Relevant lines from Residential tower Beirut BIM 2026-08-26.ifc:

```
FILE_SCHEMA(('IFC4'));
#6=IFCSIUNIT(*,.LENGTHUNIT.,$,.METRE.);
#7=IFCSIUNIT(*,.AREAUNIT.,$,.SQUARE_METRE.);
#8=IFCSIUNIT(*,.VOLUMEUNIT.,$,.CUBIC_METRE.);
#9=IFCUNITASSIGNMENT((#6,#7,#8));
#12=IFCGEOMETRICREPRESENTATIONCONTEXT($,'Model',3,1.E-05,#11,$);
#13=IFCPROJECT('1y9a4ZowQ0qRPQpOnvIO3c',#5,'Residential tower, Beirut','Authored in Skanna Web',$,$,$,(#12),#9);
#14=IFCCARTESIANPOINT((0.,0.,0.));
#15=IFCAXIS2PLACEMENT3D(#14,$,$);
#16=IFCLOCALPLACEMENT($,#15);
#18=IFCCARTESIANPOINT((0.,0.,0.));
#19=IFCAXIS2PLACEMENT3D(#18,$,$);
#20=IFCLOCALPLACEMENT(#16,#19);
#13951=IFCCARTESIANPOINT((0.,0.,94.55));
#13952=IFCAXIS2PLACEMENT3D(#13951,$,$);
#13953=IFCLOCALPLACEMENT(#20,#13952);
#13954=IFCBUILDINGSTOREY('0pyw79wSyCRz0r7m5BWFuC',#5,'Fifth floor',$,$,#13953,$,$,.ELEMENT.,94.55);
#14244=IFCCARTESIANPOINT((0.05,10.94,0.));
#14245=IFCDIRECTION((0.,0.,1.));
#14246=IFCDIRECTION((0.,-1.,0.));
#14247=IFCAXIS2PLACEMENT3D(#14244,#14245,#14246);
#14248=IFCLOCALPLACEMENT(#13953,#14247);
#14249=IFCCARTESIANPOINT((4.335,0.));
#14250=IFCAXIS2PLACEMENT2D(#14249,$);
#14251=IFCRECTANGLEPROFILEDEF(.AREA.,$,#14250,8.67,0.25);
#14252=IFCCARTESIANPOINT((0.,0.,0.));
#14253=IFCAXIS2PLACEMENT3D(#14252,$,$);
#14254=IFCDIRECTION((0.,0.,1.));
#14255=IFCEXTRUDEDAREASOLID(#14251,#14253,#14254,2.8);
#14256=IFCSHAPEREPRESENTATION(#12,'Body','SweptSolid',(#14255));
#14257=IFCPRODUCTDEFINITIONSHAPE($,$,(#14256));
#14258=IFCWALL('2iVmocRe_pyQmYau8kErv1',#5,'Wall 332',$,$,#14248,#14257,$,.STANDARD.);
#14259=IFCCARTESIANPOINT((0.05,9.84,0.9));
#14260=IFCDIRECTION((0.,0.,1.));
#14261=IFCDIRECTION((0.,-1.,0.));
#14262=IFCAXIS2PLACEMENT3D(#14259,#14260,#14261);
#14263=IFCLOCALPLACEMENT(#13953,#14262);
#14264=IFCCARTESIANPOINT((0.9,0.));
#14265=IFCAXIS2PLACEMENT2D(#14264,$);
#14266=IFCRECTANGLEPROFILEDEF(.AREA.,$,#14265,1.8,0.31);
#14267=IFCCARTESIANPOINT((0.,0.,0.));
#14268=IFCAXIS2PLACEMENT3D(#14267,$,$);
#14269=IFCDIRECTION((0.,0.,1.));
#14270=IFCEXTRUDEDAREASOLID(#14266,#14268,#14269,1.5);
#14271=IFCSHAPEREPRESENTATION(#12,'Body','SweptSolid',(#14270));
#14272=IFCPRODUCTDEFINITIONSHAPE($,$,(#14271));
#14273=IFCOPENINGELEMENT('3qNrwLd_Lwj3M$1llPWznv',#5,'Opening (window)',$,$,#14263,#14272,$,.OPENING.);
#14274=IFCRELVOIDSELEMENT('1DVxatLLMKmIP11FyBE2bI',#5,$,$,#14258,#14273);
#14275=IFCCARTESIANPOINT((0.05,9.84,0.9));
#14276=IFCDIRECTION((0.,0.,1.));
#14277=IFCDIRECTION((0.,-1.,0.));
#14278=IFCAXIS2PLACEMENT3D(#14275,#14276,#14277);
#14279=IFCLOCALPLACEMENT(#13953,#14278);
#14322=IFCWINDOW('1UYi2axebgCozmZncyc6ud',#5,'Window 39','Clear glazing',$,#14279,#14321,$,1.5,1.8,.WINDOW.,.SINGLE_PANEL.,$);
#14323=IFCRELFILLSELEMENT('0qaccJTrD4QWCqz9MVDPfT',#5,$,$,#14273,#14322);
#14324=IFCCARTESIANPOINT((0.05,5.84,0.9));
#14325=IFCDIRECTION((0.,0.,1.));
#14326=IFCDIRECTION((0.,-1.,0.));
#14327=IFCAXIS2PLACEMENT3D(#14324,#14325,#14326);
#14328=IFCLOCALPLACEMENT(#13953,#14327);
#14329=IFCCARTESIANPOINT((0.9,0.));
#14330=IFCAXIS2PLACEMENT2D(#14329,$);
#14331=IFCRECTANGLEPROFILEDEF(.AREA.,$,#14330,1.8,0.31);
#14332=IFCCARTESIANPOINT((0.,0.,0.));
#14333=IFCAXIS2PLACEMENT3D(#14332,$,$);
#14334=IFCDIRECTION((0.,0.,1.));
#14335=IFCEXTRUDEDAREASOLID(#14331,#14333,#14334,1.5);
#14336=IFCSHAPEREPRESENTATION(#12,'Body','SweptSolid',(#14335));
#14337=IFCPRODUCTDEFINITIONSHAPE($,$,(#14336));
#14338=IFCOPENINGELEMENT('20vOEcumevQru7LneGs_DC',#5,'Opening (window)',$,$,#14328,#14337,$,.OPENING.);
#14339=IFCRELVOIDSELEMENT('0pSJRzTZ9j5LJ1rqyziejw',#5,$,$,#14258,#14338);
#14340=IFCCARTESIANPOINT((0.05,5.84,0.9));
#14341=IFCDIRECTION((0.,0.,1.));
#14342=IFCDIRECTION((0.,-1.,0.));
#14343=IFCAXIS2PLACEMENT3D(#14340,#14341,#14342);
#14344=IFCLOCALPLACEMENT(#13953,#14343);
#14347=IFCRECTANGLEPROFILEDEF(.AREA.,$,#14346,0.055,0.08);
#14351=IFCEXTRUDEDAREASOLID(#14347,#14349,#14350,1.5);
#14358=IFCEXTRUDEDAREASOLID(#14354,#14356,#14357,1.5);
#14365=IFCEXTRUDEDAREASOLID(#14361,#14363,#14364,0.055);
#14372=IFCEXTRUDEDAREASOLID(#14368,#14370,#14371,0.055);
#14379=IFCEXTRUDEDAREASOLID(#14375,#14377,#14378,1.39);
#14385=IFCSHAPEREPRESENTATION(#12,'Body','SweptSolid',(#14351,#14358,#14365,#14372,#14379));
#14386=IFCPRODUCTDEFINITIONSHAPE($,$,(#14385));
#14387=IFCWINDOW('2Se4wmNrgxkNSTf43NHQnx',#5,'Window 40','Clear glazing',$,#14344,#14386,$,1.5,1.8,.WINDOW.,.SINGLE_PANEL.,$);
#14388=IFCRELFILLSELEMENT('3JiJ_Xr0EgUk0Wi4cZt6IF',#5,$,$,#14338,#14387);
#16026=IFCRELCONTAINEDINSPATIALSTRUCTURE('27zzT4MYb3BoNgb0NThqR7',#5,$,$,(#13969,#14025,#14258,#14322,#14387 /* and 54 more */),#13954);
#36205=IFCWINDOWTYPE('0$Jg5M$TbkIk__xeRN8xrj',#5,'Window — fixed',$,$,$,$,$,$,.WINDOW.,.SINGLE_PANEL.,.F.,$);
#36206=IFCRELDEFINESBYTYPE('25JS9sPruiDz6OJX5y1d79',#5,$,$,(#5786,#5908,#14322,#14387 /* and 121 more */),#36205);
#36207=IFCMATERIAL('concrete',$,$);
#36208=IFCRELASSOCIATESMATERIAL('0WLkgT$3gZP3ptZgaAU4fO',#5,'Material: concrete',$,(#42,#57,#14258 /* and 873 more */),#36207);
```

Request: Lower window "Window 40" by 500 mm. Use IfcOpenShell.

```python
import numpy as np
import ifcopenshell
import ifcopenshell.api.geometry
import ifcopenshell.util.placement
import ifcopenshell.util.unit

model = ifcopenshell.open("Residential tower Beirut BIM 2026-08-26.ifc")
unit_scale = ifcopenshell.util.unit.calculate_unit_scale(model)

window = model.by_guid("2Se4wmNrgxkNSTf43NHQnx")
opening = window.FillsVoids[0].RelatingOpeningElement
dz = -0.5 / unit_scale

shift = np.array([0.0, 0.0, dz])
# The window is not placed relative to its opening, so move both.
for product in (opening, window):
    matrix = ifcopenshell.util.placement.get_local_placement(product.ObjectPlacement)
    matrix[:3, 3] += shift
    ifcopenshell.api.geometry.edit_object_placement(model, product=product, matrix=matrix, is_si=False)

print(f"moved by {dz * unit_scale:+.3f} m")

model.write("Residential tower Beirut BIM 2026-08-26_updated.ifc")
```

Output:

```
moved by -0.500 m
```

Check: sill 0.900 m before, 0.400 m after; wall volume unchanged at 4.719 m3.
